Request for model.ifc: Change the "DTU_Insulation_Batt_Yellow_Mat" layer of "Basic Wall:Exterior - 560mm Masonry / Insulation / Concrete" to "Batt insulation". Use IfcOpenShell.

First a look at what the model holds.

```python
import ifcopenshell
import ifcopenshell.util.element

model = ifcopenshell.open("model.ifc")
print(model.schema)
for layer_set in model.by_type("IfcMaterialLayerSet"):
    if layer_set.LayerSetName == "Basic Wall:Exterior - 560mm Masonry / Insulation / Concrete":
        for layer in layer_set.MaterialLayers:
            print(layer.id(), layer.Material and layer.Material.Name, layer.LayerThickness, sep=" | ")
        print(len(ifcopenshell.util.element.get_elements_by_material(model, layer_set)), "elements and types use it")
print(sorted(m.Name for m in model.by_type("IfcMaterial") if m.Name)[:60])
```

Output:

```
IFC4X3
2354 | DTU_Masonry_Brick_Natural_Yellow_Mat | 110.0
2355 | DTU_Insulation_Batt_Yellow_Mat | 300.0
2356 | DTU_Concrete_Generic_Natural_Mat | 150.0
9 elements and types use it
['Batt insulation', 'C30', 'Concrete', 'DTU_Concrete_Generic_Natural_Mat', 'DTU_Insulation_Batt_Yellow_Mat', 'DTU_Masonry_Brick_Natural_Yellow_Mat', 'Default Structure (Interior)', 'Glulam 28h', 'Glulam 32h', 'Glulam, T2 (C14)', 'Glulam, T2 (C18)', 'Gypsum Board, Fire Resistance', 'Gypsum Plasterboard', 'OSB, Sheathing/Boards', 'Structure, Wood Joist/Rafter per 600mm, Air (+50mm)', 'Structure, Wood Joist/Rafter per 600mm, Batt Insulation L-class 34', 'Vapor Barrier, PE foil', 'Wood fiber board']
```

```python
import ifcopenshell
import ifcopenshell.api.material

model = ifcopenshell.open("model.ifc")

layer_set = next(s for s in model.by_type("IfcMaterialLayerSet") if s.LayerSetName == "Basic Wall:Exterior - 560mm Masonry / Insulation / Concrete")
layer = next(l for l in layer_set.MaterialLayers if l.Material and l.Material.Name == "DTU_Insulation_Batt_Yellow_Mat")
material = next(m for m in model.by_type("IfcMaterial") if m.Name == "Batt insulation")

# Point this one layer at the other material; renaming the old one would change it everywhere.
ifcopenshell.api.material.edit_layer(model, layer=layer, attributes={"Name": material.Name}, material=material)

print([l.Material.Name if l.Material else None for l in layer_set.MaterialLayers])

model.write("model_updated.ifc")
```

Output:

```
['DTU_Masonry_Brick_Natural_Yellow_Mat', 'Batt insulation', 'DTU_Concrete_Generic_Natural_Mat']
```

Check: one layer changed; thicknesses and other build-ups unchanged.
